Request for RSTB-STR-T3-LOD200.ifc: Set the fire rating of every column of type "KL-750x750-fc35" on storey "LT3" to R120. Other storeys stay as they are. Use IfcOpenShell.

First a look at what the model holds.

```python
import ifcopenshell
import ifcopenshell.util.element

model = ifcopenshell.open("RSTB-STR-T3-LOD200.ifc")
print(model.schema)
storey = next(s for s in model.by_type("IfcBuildingStorey") if s.Name == "LT3")
columns = [e for e in ifcopenshell.util.element.get_decomposition(storey) if e.is_a("IfcColumn")]
seen = {}
for e in columns:
    element_type = ifcopenshell.util.element.get_type(e)
    key = (element_type.Name if element_type != e and element_type else None, ifcopenshell.util.element.get_pset(e, "Pset_ColumnCommon", "FireRating"))
    seen[key] = seen.get(key, 0) + 1
for (name, value), count in sorted(seen.items(), key=str):
    print(count, "x", name, "|", value)
```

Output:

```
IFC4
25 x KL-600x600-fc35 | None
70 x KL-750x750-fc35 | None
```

```python
import ifcopenshell
import ifcopenshell.api.pset
import ifcopenshell.util.element

model = ifcopenshell.open("RSTB-STR-T3-LOD200.ifc")

storey = next(s for s in model.by_type("IfcBuildingStorey") if s.Name == "LT3")
columns = [e for e in ifcopenshell.util.element.get_decomposition(storey) if e.is_a("IfcColumn")]

count = 0
for e in columns:
    element_type = ifcopenshell.util.element.get_type(e)
    if element_type in (None, e) or element_type.Name != "KL-750x750-fc35":
        continue
    # add_pset returns the element's existing set when there is one.
    pset = ifcopenshell.api.pset.add_pset(model, product=e, name="Pset_ColumnCommon")
    ifcopenshell.api.pset.edit_pset(model, pset=pset, properties={"FireRating": "R120"})
    count += 1

print(count, "columns updated")

model.write("RSTB-STR-T3-LOD200_updated.ifc")
```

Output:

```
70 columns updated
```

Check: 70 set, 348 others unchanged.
